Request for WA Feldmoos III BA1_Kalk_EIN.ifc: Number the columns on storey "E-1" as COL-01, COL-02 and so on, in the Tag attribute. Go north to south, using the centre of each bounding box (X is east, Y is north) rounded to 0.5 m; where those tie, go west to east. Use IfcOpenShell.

First a look at what the model holds.

```python
import ifcopenshell
import ifcopenshell.util.element
import ifcopenshell.util.placement

model = ifcopenshell.open("WA Feldmoos III BA1_Kalk_EIN.ifc")
print(model.schema)
storey = next(s for s in model.by_type("IfcBuildingStorey") if s.Name == "E-1")
columns = [e for e in ifcopenshell.util.element.get_decomposition(storey) if e.is_a("IfcColumn")]
for e in sorted(columns, key=lambda e: e.id()):
    origin = ifcopenshell.util.placement.get_local_placement(e.ObjectPlacement)[:3, 3]
    print(e.id(), e.Tag, e.Name, origin.round(2) + 0.0, sep=" | ")
```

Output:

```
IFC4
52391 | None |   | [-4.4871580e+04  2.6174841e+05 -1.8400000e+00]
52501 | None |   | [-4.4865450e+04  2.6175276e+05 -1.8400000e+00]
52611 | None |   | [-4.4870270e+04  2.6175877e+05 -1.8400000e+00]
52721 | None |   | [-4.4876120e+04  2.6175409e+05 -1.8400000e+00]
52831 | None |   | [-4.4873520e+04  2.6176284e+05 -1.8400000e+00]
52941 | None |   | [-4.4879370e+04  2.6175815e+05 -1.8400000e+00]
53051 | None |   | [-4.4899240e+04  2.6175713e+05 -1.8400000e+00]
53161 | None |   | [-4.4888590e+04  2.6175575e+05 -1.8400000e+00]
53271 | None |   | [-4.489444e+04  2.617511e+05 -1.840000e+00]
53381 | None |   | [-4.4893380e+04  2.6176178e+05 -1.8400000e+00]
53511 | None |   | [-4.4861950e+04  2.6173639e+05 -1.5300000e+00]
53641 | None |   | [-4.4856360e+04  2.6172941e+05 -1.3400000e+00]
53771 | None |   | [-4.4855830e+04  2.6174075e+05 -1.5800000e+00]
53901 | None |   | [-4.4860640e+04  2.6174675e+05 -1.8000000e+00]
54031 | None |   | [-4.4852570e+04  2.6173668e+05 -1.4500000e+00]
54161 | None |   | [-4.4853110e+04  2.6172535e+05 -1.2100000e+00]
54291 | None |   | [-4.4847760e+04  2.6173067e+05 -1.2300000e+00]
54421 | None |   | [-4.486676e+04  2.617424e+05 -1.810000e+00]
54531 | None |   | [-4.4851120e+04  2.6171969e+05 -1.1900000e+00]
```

```python
import ifcopenshell
import ifcopenshell.geom
import ifcopenshell.util.element
import ifcopenshell.util.shape

model = ifcopenshell.open("WA Feldmoos III BA1_Kalk_EIN.ifc")
settings = ifcopenshell.geom.settings()
settings.set("use-world-coords", True)


def centre(element):
    shape = ifcopenshell.geom.create_shape(settings, element)
    return ifcopenshell.util.shape.get_bbox_centroid(shape.geometry)


storey = next(s for s in model.by_type("IfcBuildingStorey") if s.Name == "E-1")
columns = [e for e in ifcopenshell.util.element.get_decomposition(storey) if e.is_a("IfcColumn")]

# Insertion points can sit at a corner or the storey origin, so sort by the geometry (in metres).
centres = {e: centre(e) for e in columns}
columns.sort(key=lambda e: (-round(centres[e][1] / 0.5), centres[e][0]))

for i, e in enumerate(columns, start=1):
    number = f"COL-{i:02d}"
    e.Tag = number
    print(e.id(), number)

model.write("WA Feldmoos III BA1_Kalk_EIN_updated.ifc")
```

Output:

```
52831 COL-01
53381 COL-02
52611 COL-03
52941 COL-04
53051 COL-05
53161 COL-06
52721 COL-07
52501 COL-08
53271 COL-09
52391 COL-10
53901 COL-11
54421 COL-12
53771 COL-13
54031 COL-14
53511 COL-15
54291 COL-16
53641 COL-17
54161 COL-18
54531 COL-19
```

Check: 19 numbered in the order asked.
